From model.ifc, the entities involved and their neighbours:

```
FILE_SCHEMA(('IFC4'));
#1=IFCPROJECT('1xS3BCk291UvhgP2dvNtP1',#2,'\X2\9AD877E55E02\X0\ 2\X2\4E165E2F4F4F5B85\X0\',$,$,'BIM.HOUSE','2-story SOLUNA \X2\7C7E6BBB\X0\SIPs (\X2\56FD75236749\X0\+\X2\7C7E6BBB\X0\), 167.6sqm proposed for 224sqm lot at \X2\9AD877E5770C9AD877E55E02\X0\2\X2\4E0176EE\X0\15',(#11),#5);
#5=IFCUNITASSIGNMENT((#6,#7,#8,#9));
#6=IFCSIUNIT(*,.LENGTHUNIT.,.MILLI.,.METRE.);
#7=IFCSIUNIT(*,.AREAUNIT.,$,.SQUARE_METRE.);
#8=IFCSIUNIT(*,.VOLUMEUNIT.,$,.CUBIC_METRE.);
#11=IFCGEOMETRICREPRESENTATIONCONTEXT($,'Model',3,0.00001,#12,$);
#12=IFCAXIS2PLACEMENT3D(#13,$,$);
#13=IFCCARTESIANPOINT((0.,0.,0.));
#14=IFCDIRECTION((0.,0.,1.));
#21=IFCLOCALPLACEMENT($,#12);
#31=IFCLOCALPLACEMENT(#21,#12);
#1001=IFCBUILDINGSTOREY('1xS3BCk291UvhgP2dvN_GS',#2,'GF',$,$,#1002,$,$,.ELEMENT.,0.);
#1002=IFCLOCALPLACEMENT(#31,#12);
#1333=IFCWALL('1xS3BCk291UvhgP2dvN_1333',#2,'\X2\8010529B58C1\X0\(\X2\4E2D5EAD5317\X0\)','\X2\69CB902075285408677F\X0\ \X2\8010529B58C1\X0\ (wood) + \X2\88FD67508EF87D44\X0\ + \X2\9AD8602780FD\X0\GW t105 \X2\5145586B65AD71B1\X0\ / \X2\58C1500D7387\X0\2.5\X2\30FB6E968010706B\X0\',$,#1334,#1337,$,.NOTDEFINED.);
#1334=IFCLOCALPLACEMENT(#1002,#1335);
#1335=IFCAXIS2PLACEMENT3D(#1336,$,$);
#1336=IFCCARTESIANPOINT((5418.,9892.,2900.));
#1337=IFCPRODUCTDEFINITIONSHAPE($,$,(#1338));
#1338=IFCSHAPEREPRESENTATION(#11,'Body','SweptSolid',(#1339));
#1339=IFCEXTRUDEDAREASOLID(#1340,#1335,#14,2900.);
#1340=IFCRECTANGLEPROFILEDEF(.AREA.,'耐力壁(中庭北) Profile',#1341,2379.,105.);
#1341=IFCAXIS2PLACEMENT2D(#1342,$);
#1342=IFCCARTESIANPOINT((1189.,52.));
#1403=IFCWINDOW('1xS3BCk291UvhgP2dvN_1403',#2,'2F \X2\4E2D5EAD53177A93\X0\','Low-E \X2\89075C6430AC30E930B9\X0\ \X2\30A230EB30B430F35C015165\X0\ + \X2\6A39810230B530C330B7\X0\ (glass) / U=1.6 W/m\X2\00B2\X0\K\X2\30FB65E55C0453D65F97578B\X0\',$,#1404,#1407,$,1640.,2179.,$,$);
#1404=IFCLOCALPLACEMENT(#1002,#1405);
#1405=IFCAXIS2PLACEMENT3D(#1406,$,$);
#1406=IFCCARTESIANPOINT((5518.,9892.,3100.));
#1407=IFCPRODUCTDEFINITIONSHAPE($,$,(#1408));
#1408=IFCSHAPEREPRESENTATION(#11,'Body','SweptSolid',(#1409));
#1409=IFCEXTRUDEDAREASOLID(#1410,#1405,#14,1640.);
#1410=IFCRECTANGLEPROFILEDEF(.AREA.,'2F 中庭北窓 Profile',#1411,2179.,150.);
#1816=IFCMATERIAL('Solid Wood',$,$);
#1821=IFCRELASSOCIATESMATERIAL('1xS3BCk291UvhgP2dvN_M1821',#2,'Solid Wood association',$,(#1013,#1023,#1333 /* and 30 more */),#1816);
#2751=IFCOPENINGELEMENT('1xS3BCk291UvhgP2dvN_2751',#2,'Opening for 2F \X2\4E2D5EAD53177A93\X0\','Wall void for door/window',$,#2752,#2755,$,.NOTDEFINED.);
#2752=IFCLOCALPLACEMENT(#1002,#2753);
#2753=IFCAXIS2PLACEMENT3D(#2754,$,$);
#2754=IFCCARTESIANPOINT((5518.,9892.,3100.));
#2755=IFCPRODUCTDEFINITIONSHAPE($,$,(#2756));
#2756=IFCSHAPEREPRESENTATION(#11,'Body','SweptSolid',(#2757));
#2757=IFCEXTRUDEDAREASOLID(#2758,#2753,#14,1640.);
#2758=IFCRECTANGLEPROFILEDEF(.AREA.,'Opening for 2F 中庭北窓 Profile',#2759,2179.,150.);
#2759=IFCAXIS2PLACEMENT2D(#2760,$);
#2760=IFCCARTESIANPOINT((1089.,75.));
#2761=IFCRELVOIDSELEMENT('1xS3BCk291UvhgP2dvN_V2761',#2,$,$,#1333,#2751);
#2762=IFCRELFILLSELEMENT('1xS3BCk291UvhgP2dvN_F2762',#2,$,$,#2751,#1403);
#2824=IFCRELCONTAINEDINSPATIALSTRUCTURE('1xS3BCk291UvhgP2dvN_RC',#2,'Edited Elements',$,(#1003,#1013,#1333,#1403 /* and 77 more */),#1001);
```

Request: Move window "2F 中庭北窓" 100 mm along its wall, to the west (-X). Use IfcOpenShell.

```python
import ifcopenshell
import ifcopenshell.api.geometry
import ifcopenshell.util.placement
import ifcopenshell.util.unit

model = ifcopenshell.open("model.ifc")
unit_scale = ifcopenshell.util.unit.calculate_unit_scale(model)

window = model.by_id(1403)
opening = window.FillsVoids[0].RelatingOpeningElement
wall = opening.VoidsElements[0].RelatingBuildingElement

wall_matrix = ifcopenshell.util.placement.get_local_placement(wall.ObjectPlacement)
shift = wall_matrix[:3, 0] * -0.1 / unit_scale
before = ifcopenshell.util.placement.get_local_placement(window.ObjectPlacement)[:3, 3].copy()

# The window is not placed relative to its opening, so move both.
for product in (opening, window):
    matrix = ifcopenshell.util.placement.get_local_placement(product.ObjectPlacement)
    matrix[:3, 3] += shift
    ifcopenshell.api.geometry.edit_object_placement(model, product=product, matrix=matrix, is_si=False)

after = ifcopenshell.util.placement.get_local_placement(window.ObjectPlacement)[:3, 3]
print("window moved by", (after - before).round(3) + 0.0)

model.write("model_v2.ifc")
```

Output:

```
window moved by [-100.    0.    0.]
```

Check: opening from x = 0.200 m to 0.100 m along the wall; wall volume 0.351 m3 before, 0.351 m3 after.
